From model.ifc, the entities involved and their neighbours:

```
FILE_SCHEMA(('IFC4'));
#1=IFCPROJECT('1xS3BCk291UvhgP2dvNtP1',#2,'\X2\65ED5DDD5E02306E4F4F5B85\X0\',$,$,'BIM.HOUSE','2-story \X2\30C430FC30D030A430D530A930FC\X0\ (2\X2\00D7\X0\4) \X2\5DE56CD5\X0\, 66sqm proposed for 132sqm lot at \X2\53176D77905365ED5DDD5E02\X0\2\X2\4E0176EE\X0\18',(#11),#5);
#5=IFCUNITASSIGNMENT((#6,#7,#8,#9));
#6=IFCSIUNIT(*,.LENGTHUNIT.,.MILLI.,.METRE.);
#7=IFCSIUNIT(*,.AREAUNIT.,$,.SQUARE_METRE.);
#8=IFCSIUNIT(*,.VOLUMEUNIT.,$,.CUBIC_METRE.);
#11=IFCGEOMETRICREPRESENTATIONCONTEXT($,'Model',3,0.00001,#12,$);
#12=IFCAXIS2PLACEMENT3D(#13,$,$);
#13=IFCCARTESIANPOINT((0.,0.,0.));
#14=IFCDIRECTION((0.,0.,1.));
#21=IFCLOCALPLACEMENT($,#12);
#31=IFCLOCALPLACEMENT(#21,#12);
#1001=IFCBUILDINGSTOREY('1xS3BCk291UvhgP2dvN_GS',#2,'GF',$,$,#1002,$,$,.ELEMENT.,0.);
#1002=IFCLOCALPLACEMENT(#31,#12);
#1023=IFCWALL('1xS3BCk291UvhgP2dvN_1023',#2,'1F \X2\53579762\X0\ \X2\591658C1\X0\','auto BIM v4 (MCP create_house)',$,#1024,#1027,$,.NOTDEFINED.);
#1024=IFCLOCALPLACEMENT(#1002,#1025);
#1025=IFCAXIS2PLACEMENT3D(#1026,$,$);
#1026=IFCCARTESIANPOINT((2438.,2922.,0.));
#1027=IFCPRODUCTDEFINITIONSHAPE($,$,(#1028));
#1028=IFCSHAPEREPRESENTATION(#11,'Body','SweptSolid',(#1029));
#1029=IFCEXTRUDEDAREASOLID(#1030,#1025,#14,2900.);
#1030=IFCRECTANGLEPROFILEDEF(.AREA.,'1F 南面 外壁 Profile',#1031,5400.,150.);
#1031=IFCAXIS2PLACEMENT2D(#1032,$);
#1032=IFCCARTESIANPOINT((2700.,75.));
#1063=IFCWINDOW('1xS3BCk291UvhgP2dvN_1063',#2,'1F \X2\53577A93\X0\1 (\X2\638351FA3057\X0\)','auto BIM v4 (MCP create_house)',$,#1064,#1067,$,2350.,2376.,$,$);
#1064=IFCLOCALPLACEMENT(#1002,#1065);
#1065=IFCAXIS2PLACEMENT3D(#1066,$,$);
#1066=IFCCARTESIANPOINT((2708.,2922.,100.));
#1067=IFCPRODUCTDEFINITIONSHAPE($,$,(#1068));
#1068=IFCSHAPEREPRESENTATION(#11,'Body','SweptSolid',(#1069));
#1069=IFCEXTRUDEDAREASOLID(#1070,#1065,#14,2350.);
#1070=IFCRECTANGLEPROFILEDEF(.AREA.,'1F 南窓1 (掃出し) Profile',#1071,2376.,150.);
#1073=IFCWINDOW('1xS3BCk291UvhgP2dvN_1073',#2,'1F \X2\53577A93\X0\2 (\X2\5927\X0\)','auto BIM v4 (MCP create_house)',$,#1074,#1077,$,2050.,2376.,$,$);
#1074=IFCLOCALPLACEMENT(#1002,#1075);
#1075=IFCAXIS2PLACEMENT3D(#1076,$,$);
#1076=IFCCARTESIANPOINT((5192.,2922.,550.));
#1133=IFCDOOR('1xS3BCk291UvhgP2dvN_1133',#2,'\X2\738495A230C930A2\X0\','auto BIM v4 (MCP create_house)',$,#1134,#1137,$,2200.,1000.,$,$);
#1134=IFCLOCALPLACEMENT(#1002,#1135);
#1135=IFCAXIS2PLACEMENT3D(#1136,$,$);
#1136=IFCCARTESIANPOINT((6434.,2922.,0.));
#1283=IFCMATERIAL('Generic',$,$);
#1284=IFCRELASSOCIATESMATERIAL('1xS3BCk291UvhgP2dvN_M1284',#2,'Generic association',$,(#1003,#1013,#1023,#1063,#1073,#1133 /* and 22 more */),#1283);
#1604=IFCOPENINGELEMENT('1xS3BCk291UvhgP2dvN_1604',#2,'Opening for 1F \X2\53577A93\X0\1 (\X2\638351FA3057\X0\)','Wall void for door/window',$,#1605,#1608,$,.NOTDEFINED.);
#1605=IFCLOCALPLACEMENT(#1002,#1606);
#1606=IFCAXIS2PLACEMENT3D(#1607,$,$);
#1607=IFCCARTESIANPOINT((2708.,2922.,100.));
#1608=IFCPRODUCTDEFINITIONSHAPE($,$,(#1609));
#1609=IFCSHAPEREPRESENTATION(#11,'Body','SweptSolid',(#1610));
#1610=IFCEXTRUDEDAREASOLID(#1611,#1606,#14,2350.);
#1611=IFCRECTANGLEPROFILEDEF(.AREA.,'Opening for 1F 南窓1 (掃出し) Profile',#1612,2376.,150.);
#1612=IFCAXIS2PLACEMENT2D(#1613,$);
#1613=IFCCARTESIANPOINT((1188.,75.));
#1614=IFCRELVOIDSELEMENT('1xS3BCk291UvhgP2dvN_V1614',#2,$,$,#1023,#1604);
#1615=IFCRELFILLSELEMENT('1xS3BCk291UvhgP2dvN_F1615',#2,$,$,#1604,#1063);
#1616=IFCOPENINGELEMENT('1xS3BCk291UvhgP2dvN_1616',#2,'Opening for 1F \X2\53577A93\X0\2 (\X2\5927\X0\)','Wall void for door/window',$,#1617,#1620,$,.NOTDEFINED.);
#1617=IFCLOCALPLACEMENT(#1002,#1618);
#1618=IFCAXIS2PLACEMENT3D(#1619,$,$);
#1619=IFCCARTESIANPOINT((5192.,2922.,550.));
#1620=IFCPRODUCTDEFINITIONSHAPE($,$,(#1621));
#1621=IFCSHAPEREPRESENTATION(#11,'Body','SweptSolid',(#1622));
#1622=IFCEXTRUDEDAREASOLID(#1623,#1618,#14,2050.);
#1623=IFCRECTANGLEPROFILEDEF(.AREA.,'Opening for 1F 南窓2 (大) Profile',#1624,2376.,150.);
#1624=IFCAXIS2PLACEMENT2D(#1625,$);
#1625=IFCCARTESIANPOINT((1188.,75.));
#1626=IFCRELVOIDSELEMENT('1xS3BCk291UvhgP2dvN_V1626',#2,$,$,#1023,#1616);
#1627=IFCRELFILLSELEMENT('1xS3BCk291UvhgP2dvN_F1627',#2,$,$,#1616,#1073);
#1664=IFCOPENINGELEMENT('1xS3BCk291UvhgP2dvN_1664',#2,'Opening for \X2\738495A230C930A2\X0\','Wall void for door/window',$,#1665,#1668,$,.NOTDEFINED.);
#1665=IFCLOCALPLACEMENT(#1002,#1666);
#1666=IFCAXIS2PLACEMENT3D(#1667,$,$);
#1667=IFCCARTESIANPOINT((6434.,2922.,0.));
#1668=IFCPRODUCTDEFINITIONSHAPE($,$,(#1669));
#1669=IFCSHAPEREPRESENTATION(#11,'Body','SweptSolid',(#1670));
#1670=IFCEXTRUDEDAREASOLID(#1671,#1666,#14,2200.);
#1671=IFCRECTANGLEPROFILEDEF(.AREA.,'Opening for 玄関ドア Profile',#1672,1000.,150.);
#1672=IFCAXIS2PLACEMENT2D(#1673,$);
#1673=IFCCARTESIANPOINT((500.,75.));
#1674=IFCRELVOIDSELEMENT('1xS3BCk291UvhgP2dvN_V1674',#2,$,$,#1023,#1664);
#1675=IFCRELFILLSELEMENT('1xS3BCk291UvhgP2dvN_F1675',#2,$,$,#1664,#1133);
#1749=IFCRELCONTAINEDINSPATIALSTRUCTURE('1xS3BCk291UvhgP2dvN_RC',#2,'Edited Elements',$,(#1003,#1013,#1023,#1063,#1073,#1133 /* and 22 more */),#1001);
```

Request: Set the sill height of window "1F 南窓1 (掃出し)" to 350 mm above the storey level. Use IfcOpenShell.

```python
import numpy as np
import ifcopenshell
import ifcopenshell.api.geometry
import ifcopenshell.geom
import ifcopenshell.util.element
import ifcopenshell.util.placement
import ifcopenshell.util.shape
import ifcopenshell.util.unit

model = ifcopenshell.open("model.ifc")
unit_scale = ifcopenshell.util.unit.calculate_unit_scale(model)

window = model.by_guid("1xS3BCk291UvhgP2dvN_1063")
opening = window.FillsVoids[0].RelatingOpeningElement
storey = ifcopenshell.util.element.get_container(window, ifc_class="IfcBuildingStorey")
level = ifcopenshell.util.placement.get_local_placement(storey.ObjectPlacement)[2, 3]

# The opening's origin need not be at the sill, so measure its lowest point.
shape = ifcopenshell.geom.create_shape(ifcopenshell.geom.settings(), opening)
bottom = ifcopenshell.util.shape.get_shape_bottom_elevation(shape, shape.geometry) / unit_scale
dz = level + 350.0 - bottom

shift = np.array([0.0, 0.0, dz])
# The window is not placed relative to its opening, so move both.
for product in (opening, window):
    matrix = ifcopenshell.util.placement.get_local_placement(product.ObjectPlacement)
    matrix[:3, 3] += shift
    ifcopenshell.api.geometry.edit_object_placement(model, product=product, matrix=matrix, is_si=False)

print(f"moved by {dz * unit_scale:+.3f} m")

model.write("model_edited.ifc")
```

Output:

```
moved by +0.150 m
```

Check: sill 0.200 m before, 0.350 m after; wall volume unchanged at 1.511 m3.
